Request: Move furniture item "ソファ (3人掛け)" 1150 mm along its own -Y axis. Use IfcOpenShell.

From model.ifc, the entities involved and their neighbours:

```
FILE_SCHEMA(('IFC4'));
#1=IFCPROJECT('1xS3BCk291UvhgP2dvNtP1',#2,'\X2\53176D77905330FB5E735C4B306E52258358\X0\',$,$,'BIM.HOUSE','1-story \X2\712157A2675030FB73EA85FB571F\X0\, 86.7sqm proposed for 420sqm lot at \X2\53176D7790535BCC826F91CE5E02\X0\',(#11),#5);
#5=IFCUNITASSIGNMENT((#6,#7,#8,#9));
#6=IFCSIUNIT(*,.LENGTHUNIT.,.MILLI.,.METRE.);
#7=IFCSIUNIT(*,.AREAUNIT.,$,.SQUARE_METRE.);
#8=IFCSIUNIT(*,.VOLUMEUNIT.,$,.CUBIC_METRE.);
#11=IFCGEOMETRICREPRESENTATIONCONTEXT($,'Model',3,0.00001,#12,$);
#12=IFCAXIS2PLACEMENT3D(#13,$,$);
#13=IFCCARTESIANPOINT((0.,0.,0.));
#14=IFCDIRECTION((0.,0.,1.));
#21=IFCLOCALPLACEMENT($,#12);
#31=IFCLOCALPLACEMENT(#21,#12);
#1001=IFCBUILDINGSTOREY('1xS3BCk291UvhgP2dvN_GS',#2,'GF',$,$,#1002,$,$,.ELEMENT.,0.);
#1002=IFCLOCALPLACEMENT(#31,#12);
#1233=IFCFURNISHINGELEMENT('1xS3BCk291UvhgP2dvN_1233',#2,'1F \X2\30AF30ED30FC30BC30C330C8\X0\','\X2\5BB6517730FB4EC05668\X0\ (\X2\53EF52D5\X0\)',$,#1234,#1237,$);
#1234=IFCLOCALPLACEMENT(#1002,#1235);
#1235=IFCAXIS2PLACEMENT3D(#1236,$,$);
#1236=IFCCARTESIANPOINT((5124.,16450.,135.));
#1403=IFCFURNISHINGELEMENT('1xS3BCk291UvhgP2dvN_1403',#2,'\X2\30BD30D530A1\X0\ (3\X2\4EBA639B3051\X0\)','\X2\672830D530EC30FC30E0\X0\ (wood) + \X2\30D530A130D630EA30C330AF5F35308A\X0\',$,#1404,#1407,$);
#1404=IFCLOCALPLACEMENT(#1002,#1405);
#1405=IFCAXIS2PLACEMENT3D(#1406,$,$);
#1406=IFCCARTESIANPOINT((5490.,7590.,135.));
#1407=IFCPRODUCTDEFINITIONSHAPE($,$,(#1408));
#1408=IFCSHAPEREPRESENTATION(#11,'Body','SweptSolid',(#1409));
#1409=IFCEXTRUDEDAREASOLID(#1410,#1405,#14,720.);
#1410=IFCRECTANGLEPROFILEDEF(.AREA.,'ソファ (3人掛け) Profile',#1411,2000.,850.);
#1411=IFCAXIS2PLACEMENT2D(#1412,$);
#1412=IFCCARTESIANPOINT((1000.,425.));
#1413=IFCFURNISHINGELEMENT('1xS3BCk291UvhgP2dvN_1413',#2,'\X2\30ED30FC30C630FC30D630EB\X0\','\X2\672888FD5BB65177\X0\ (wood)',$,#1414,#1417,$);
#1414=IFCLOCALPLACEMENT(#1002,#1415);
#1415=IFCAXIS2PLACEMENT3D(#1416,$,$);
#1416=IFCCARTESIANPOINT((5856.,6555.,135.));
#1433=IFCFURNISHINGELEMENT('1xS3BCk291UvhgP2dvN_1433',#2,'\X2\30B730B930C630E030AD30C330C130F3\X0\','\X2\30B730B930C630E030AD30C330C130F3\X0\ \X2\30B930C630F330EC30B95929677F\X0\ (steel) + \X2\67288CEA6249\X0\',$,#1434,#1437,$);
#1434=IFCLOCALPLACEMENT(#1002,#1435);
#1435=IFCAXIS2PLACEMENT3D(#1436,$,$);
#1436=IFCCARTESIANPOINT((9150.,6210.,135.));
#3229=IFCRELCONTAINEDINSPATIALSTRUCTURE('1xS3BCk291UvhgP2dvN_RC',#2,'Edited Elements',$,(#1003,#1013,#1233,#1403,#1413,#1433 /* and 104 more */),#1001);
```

```python
import ifcopenshell
import ifcopenshell.api.geometry
import ifcopenshell.util.placement
import ifcopenshell.util.unit

model = ifcopenshell.open("model.ifc")
unit_scale = ifcopenshell.util.unit.calculate_unit_scale(model)

item = model.by_guid("1xS3BCk291UvhgP2dvN_1403")
matrix = ifcopenshell.util.placement.get_local_placement(item.ObjectPlacement)
matrix[:3, 3] -= matrix[:3, 1] * 1.15 / unit_scale
ifcopenshell.api.geometry.edit_object_placement(model, product=item, matrix=matrix, is_si=False)

print(ifcopenshell.util.placement.get_local_placement(item.ObjectPlacement).round(3) + 0.0)

model.write("model_updated.ifc")
```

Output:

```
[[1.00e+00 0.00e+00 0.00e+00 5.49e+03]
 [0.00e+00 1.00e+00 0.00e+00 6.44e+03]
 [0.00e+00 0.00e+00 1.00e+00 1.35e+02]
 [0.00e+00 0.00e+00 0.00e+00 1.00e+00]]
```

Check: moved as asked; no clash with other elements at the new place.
